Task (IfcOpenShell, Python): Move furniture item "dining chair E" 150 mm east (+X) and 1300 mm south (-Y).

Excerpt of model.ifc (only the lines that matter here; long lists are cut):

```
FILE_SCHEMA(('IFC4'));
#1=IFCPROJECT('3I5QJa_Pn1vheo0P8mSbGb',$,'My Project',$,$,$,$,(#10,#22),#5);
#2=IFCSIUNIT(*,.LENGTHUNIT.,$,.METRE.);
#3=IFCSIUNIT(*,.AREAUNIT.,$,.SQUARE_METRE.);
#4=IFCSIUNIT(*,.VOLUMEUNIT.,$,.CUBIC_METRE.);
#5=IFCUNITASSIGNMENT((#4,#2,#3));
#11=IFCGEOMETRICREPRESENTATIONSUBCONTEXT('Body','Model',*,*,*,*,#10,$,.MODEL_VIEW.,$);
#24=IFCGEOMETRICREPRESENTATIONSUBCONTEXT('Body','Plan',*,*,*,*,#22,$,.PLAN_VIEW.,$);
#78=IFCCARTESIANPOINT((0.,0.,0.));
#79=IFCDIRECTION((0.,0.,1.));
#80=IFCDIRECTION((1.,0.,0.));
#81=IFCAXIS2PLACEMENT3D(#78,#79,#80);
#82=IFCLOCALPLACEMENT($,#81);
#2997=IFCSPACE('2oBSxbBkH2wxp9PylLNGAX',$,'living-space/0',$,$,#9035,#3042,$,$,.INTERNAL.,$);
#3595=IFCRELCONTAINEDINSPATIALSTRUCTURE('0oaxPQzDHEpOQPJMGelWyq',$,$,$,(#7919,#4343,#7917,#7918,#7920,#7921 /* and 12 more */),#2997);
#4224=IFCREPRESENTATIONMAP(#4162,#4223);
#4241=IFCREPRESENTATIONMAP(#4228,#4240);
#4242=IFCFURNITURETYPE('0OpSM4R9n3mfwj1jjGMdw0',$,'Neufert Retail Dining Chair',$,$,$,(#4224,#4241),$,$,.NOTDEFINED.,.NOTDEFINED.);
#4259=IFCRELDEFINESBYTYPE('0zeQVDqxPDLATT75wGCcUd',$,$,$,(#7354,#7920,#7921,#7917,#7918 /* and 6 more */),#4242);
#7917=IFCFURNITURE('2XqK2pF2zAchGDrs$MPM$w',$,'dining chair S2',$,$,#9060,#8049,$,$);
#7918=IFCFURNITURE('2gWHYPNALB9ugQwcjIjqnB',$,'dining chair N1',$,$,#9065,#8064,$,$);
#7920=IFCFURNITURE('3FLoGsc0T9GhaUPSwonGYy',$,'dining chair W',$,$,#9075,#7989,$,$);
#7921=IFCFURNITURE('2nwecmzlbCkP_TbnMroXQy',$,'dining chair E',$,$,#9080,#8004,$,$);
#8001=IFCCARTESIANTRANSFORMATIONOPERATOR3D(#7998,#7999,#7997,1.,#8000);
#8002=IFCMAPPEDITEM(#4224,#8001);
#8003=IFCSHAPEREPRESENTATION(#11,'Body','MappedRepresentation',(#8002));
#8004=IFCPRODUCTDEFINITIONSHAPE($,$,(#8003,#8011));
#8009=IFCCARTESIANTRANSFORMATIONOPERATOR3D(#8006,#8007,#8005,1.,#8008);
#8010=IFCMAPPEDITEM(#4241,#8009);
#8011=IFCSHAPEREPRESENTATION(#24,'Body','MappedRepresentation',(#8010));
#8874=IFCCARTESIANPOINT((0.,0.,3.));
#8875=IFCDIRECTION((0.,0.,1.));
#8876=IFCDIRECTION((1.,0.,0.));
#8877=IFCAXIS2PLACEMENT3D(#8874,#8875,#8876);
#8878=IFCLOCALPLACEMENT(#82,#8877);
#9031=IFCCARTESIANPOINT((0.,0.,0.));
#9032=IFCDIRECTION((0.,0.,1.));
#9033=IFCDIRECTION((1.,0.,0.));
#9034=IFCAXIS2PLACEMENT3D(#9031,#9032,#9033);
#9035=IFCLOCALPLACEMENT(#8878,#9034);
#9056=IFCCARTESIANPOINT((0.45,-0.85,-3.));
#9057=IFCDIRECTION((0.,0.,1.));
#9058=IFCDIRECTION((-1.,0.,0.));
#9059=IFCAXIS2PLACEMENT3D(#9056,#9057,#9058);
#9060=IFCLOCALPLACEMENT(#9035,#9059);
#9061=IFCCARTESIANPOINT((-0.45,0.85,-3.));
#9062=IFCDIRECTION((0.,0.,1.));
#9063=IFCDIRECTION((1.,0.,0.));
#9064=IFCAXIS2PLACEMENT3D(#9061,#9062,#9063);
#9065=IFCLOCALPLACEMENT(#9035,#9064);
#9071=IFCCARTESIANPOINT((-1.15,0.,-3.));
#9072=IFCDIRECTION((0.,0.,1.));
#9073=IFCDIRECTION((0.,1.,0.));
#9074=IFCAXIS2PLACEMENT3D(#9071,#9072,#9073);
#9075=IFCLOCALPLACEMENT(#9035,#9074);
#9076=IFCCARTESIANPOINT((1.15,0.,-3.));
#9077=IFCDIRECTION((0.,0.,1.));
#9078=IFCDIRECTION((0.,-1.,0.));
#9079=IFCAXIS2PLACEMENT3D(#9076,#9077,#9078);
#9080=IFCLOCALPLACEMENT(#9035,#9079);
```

```python
import ifcopenshell
import ifcopenshell.api.geometry
import ifcopenshell.util.placement
import ifcopenshell.util.unit

model = ifcopenshell.open("model.ifc")
unit_scale = ifcopenshell.util.unit.calculate_unit_scale(model)

item = model.by_guid("2nwecmzlbCkP_TbnMroXQy")
matrix = ifcopenshell.util.placement.get_local_placement(item.ObjectPlacement)
matrix[0, 3] += 0.15 / unit_scale
matrix[1, 3] -= 1.3 / unit_scale
ifcopenshell.api.geometry.edit_object_placement(model, product=item, matrix=matrix, is_si=False)

print(ifcopenshell.util.placement.get_local_placement(item.ObjectPlacement).round(3) + 0.0)

model.write("model-out.ifc")
```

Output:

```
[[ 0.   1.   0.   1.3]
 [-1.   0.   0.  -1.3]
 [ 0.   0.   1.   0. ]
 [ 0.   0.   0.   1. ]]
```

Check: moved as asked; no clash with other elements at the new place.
